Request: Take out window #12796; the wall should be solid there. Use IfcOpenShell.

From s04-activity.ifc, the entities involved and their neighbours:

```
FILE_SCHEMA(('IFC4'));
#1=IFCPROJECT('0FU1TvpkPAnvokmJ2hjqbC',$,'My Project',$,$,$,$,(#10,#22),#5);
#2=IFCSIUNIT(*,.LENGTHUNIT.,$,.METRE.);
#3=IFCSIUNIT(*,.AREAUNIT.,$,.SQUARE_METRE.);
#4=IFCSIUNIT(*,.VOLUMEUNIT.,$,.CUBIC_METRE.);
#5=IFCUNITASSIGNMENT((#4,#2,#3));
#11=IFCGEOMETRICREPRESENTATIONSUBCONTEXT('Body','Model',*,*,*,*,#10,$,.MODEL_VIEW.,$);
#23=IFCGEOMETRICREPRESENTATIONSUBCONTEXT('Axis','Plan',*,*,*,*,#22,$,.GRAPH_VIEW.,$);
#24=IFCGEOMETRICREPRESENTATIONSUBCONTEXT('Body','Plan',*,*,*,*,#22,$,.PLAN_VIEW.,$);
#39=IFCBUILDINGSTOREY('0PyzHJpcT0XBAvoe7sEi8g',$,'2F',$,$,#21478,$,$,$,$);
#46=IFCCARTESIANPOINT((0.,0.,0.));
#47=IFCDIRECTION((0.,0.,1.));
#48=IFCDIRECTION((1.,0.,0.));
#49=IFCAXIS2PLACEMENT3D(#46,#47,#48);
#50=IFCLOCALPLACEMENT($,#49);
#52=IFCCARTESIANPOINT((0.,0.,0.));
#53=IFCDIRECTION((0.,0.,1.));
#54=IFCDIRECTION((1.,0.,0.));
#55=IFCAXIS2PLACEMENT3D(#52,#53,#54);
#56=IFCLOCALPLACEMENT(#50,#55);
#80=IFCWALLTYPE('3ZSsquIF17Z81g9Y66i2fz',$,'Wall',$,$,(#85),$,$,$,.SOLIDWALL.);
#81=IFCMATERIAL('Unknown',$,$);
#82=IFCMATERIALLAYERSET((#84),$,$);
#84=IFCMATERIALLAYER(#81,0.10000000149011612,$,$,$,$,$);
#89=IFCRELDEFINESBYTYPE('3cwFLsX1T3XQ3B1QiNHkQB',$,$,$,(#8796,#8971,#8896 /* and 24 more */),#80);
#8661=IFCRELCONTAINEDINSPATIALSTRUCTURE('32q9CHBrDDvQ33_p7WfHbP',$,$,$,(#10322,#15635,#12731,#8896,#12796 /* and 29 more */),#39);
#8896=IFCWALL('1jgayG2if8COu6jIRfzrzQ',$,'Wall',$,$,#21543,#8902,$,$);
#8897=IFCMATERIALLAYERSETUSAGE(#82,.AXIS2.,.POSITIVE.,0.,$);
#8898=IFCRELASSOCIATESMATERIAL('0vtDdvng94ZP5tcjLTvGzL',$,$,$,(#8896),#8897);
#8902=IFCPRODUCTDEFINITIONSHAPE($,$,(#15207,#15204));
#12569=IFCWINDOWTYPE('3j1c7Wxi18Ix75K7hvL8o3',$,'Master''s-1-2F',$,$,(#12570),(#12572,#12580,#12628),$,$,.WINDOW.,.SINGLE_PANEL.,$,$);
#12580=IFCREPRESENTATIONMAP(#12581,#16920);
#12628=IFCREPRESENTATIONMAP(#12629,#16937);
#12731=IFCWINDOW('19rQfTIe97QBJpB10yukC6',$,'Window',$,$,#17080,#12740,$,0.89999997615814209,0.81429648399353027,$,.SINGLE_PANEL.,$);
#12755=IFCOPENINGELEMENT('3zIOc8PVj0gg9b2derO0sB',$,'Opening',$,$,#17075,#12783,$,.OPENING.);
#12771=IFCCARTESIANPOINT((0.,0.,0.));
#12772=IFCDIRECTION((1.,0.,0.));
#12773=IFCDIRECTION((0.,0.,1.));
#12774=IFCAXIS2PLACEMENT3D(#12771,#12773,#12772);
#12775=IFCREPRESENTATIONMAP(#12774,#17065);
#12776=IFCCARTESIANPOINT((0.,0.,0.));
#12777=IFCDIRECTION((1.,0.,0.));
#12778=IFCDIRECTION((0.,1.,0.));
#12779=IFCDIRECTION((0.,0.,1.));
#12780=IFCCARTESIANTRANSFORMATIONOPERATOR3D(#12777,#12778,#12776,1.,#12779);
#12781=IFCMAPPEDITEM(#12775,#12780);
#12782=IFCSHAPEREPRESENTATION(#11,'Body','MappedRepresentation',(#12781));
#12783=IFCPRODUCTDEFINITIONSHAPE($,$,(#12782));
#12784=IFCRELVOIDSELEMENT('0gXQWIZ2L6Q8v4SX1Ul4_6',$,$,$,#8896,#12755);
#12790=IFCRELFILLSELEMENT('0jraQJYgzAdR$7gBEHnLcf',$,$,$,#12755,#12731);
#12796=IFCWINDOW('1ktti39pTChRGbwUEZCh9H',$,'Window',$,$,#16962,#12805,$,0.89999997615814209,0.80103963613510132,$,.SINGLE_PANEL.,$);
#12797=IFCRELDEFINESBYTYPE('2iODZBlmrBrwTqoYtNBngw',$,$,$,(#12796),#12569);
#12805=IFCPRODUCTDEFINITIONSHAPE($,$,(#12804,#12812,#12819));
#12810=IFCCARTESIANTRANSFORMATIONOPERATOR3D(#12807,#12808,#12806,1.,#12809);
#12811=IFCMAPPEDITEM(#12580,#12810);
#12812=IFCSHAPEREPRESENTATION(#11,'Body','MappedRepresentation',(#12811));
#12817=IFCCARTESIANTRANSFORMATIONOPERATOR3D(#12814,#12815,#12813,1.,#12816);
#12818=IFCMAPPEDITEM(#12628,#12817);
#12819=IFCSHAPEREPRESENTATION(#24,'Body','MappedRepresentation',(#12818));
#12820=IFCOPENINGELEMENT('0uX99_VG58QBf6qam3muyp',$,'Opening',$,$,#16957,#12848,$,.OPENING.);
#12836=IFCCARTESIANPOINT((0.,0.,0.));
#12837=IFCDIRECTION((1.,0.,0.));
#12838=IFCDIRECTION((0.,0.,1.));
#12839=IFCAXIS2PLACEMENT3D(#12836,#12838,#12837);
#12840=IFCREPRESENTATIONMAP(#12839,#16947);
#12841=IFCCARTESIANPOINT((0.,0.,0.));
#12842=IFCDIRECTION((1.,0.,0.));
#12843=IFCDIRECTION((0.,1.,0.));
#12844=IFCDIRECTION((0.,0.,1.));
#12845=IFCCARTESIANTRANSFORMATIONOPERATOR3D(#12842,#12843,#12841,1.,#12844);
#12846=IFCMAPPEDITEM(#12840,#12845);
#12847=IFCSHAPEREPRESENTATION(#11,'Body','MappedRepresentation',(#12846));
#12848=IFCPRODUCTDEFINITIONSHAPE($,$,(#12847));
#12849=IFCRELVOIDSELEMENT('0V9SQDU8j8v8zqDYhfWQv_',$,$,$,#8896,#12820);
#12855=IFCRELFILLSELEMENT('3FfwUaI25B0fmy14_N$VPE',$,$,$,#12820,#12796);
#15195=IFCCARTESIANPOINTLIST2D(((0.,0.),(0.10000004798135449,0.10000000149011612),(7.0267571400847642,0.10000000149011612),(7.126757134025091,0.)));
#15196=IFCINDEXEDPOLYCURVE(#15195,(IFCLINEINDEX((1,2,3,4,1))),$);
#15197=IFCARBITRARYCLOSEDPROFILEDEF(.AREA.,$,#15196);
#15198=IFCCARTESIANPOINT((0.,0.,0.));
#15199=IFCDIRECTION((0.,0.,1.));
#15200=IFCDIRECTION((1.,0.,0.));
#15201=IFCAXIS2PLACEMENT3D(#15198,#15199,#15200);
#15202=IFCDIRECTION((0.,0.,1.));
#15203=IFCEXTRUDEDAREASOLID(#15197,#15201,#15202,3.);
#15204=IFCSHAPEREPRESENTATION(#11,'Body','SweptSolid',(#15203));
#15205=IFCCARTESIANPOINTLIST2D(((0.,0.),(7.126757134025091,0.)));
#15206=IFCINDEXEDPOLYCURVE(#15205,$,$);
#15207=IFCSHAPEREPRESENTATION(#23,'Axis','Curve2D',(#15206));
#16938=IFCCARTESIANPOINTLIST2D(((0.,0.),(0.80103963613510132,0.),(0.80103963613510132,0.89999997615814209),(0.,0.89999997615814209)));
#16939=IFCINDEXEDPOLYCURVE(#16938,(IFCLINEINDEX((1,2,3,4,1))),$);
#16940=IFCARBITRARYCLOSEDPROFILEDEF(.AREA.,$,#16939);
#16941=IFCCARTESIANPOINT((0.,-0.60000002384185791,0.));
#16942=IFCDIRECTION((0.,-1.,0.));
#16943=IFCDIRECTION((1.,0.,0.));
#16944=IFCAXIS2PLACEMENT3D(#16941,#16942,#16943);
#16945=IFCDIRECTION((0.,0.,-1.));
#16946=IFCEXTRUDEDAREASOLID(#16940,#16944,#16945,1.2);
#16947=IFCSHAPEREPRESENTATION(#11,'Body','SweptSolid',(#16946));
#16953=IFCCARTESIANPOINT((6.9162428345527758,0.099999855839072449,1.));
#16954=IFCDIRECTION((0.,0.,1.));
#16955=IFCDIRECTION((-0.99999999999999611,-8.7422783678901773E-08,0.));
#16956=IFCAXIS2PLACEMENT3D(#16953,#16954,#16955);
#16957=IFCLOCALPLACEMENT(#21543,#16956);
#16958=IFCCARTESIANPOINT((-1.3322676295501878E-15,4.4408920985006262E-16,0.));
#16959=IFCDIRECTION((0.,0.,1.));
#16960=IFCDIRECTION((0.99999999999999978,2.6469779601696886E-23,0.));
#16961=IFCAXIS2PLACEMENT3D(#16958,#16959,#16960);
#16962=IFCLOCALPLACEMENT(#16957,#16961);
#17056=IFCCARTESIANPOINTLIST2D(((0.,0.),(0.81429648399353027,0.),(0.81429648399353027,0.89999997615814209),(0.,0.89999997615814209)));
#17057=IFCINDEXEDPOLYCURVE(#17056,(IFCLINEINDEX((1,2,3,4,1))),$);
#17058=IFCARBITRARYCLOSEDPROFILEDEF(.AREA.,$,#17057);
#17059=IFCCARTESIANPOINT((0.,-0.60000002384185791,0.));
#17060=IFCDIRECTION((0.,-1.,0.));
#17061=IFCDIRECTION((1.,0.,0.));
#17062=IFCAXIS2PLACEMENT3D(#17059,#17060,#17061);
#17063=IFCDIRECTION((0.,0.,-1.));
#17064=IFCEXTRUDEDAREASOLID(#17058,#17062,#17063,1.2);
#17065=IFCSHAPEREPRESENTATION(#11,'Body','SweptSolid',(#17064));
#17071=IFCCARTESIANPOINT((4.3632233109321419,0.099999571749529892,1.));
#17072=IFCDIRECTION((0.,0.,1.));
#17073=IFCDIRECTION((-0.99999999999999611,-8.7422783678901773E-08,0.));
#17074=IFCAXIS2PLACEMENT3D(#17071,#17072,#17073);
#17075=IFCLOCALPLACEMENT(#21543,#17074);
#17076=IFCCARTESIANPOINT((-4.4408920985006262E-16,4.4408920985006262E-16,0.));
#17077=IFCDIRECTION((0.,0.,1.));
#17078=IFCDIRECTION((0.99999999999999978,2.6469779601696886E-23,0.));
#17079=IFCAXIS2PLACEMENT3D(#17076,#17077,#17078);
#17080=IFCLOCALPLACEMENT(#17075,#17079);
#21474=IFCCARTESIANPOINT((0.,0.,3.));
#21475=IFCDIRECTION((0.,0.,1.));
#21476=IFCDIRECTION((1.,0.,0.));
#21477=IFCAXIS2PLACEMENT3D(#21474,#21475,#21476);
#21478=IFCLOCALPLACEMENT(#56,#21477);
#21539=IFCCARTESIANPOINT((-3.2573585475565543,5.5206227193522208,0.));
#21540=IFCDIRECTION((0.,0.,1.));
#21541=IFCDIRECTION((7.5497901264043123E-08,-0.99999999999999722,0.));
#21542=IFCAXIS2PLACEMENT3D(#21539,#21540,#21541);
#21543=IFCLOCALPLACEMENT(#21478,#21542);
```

```python
import ifcopenshell
import ifcopenshell.api.feature
import ifcopenshell.api.root
import ifcopenshell.geom
import ifcopenshell.util.shape

model = ifcopenshell.open("s04-activity.ifc")
settings = ifcopenshell.geom.settings()


def volume(element):
    """Net volume in cubic metres, openings subtracted."""
    shape = ifcopenshell.geom.create_shape(settings, element)
    return ifcopenshell.util.shape.get_volume(shape.geometry)


window = model.by_guid("1ktti39pTChRGbwUEZCh9H")
opening = window.FillsVoids[0].RelatingOpeningElement
wall = opening.VoidsElements[0].RelatingBuildingElement
before = volume(wall)

ifcopenshell.api.root.remove_product(model, product=window)
ifcopenshell.api.feature.remove_feature(model, feature=opening)

after = volume(wall)

print(f"wall volume {before:.3f} -> {after:.3f} m3")

model.write("s04-activity-out.ifc")
```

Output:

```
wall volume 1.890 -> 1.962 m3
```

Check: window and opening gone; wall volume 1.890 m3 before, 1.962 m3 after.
